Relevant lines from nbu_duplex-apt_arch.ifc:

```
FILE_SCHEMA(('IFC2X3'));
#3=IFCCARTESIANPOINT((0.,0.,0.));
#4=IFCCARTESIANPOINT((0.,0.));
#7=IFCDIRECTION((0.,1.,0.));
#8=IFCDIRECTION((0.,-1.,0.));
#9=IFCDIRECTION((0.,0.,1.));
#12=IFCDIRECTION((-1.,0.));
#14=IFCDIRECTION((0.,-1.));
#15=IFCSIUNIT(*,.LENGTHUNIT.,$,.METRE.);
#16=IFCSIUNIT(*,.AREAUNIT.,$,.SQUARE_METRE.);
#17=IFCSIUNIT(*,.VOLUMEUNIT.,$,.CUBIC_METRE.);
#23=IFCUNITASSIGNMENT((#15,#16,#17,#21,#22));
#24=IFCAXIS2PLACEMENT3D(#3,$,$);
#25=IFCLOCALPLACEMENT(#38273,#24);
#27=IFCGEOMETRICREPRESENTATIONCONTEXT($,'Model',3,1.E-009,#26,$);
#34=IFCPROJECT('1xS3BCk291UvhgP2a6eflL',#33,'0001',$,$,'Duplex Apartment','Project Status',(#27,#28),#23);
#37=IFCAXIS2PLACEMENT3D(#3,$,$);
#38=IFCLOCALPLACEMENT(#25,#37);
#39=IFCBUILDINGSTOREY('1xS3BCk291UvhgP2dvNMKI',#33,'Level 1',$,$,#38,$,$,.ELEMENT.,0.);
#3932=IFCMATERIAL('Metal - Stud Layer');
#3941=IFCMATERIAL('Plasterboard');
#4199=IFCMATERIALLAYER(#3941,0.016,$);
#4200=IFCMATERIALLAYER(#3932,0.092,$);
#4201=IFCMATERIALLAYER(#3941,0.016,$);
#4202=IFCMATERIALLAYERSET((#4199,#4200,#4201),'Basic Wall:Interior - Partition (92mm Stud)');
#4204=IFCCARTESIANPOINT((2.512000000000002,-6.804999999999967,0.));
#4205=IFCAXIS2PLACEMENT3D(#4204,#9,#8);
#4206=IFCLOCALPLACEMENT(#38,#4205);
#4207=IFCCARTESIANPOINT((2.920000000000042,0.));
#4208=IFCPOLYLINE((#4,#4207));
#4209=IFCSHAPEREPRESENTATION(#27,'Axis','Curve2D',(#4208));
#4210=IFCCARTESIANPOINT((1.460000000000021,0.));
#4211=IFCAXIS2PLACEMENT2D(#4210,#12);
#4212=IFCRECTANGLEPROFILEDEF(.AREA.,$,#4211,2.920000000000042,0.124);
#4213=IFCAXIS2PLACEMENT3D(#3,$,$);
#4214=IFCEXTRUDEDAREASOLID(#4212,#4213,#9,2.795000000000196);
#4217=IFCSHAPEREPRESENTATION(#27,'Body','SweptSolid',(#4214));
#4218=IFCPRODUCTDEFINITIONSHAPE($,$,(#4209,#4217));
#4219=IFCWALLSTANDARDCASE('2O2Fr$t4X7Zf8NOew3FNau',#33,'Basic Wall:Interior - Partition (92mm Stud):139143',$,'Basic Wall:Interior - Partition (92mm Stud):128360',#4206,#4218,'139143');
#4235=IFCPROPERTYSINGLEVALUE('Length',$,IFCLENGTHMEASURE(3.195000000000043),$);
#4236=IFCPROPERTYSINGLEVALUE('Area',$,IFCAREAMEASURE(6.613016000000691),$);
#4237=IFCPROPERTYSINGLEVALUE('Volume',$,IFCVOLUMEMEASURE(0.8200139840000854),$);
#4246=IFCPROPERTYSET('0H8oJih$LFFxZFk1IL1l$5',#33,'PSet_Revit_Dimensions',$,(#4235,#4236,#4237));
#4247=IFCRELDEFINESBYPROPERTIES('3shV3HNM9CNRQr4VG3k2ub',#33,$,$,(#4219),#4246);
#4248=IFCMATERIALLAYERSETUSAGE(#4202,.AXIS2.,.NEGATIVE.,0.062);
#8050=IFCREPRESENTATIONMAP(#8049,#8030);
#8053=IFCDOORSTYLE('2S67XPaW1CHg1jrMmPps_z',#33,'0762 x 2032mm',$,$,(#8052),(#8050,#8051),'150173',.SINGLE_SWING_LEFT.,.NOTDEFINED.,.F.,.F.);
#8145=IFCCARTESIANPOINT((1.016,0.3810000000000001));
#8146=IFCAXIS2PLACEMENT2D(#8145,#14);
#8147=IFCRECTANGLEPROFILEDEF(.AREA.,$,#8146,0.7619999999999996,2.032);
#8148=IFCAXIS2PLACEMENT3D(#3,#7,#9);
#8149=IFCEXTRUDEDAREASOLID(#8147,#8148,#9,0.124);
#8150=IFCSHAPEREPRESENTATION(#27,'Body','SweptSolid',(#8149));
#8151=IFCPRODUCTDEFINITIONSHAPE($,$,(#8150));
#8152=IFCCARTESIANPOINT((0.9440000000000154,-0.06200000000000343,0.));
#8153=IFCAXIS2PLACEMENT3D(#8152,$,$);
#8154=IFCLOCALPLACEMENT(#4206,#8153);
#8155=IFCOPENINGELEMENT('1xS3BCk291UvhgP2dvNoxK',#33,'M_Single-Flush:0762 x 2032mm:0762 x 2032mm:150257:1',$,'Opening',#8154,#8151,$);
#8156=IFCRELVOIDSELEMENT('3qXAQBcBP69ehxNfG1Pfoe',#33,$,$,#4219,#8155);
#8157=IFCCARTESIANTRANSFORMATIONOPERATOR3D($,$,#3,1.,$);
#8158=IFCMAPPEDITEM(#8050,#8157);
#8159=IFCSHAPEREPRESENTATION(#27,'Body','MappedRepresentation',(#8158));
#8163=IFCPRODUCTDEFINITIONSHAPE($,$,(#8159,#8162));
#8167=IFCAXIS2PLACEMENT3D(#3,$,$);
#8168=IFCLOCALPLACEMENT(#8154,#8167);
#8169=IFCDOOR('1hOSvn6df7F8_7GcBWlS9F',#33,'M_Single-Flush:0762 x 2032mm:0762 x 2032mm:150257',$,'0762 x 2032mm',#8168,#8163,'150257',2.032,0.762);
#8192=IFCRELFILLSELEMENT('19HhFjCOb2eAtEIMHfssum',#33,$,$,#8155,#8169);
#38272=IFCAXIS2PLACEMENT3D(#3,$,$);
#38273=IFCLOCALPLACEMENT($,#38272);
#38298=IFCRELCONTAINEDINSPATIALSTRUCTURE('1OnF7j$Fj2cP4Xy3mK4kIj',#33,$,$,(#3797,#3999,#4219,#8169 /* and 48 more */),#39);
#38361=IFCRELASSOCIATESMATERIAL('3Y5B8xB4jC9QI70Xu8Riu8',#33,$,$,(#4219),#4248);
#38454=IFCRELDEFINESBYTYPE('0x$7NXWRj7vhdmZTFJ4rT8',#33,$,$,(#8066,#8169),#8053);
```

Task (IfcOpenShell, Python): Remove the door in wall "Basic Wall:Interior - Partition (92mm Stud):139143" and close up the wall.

```python
import ifcopenshell
import ifcopenshell.api.feature
import ifcopenshell.api.pset
import ifcopenshell.api.root
import ifcopenshell.geom
import ifcopenshell.util.element
import ifcopenshell.util.shape
import ifcopenshell.util.unit

model = ifcopenshell.open("nbu_duplex-apt_arch.ifc")
area_scale = ifcopenshell.util.unit.calculate_unit_scale(model, "AREAUNIT")
volume_scale = ifcopenshell.util.unit.calculate_unit_scale(model, "VOLUMEUNIT")
settings = ifcopenshell.geom.settings()


def volume(element):
    """Net volume in cubic metres, openings subtracted."""
    shape = ifcopenshell.geom.create_shape(settings, element)
    return ifcopenshell.util.shape.get_volume(shape.geometry)


door = model.by_guid("1hOSvn6df7F8_7GcBWlS9F")
opening = door.FillsVoids[0].RelatingOpeningElement
wall = opening.VoidsElements[0].RelatingBuildingElement
before = volume(wall)

ifcopenshell.api.root.remove_product(model, product=door)
ifcopenshell.api.feature.remove_feature(model, feature=opening)

after = volume(wall)
thickness = 0.124  # wall thickness in metres

# Update the wall's stored quantities.
pset = model.by_id(ifcopenshell.util.element.get_pset(wall, "PSet_Revit_Dimensions", should_inherit=False)["id"])
ifcopenshell.api.pset.edit_pset(model, pset=pset, properties={
    "Area": model.create_entity("IfcAreaMeasure", after / thickness / area_scale),
    "Volume": model.create_entity("IfcVolumeMeasure", after / volume_scale),
})

print(f"wall volume {before:.3f} -> {after:.3f} m3")

model.write("nbu_duplex-apt_arch_updated.ifc")
```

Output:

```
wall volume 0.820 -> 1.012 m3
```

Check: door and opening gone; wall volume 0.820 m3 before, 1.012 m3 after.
